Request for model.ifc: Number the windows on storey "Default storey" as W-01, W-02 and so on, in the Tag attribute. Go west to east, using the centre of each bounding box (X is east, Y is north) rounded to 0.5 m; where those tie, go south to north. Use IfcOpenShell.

First a look at what the model holds.

```python
import ifcopenshell
import ifcopenshell.util.element
import ifcopenshell.util.placement

model = ifcopenshell.open("model.ifc")
print(model.schema)
storey = next(s for s in model.by_type("IfcBuildingStorey") if s.Name == "Default storey")
windows = [e for e in ifcopenshell.util.element.get_decomposition(storey) if e.is_a("IfcWindow")]
for e in sorted(windows, key=lambda e: e.id()):
    origin = ifcopenshell.util.placement.get_local_placement(e.ObjectPlacement)[:3, 3]
    print(e.id(), e.Tag, e.Name, origin.round(2) + 0.0, sep=" | ")
```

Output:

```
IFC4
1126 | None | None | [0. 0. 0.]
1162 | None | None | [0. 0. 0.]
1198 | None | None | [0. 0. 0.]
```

```python
import ifcopenshell
import ifcopenshell.geom
import ifcopenshell.util.element
import ifcopenshell.util.shape

model = ifcopenshell.open("model.ifc")
settings = ifcopenshell.geom.settings()
settings.set("use-world-coords", True)


def centre(element):
    shape = ifcopenshell.geom.create_shape(settings, element)
    return ifcopenshell.util.shape.get_bbox_centroid(shape.geometry)


storey = next(s for s in model.by_type("IfcBuildingStorey") if s.Name == "Default storey")
windows = [e for e in ifcopenshell.util.element.get_decomposition(storey) if e.is_a("IfcWindow")]

# Insertion points can sit at a corner or the storey origin, so sort by the geometry (in metres).
centres = {e: centre(e) for e in windows}
windows.sort(key=lambda e: (round(centres[e][0] / 0.5), centres[e][1]))

for i, e in enumerate(windows, start=1):
    number = f"W-{i:02d}"
    e.Tag = number
    print(e.id(), number)

model.write("model_v2.ifc")
```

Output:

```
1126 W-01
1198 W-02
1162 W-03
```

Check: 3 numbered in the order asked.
